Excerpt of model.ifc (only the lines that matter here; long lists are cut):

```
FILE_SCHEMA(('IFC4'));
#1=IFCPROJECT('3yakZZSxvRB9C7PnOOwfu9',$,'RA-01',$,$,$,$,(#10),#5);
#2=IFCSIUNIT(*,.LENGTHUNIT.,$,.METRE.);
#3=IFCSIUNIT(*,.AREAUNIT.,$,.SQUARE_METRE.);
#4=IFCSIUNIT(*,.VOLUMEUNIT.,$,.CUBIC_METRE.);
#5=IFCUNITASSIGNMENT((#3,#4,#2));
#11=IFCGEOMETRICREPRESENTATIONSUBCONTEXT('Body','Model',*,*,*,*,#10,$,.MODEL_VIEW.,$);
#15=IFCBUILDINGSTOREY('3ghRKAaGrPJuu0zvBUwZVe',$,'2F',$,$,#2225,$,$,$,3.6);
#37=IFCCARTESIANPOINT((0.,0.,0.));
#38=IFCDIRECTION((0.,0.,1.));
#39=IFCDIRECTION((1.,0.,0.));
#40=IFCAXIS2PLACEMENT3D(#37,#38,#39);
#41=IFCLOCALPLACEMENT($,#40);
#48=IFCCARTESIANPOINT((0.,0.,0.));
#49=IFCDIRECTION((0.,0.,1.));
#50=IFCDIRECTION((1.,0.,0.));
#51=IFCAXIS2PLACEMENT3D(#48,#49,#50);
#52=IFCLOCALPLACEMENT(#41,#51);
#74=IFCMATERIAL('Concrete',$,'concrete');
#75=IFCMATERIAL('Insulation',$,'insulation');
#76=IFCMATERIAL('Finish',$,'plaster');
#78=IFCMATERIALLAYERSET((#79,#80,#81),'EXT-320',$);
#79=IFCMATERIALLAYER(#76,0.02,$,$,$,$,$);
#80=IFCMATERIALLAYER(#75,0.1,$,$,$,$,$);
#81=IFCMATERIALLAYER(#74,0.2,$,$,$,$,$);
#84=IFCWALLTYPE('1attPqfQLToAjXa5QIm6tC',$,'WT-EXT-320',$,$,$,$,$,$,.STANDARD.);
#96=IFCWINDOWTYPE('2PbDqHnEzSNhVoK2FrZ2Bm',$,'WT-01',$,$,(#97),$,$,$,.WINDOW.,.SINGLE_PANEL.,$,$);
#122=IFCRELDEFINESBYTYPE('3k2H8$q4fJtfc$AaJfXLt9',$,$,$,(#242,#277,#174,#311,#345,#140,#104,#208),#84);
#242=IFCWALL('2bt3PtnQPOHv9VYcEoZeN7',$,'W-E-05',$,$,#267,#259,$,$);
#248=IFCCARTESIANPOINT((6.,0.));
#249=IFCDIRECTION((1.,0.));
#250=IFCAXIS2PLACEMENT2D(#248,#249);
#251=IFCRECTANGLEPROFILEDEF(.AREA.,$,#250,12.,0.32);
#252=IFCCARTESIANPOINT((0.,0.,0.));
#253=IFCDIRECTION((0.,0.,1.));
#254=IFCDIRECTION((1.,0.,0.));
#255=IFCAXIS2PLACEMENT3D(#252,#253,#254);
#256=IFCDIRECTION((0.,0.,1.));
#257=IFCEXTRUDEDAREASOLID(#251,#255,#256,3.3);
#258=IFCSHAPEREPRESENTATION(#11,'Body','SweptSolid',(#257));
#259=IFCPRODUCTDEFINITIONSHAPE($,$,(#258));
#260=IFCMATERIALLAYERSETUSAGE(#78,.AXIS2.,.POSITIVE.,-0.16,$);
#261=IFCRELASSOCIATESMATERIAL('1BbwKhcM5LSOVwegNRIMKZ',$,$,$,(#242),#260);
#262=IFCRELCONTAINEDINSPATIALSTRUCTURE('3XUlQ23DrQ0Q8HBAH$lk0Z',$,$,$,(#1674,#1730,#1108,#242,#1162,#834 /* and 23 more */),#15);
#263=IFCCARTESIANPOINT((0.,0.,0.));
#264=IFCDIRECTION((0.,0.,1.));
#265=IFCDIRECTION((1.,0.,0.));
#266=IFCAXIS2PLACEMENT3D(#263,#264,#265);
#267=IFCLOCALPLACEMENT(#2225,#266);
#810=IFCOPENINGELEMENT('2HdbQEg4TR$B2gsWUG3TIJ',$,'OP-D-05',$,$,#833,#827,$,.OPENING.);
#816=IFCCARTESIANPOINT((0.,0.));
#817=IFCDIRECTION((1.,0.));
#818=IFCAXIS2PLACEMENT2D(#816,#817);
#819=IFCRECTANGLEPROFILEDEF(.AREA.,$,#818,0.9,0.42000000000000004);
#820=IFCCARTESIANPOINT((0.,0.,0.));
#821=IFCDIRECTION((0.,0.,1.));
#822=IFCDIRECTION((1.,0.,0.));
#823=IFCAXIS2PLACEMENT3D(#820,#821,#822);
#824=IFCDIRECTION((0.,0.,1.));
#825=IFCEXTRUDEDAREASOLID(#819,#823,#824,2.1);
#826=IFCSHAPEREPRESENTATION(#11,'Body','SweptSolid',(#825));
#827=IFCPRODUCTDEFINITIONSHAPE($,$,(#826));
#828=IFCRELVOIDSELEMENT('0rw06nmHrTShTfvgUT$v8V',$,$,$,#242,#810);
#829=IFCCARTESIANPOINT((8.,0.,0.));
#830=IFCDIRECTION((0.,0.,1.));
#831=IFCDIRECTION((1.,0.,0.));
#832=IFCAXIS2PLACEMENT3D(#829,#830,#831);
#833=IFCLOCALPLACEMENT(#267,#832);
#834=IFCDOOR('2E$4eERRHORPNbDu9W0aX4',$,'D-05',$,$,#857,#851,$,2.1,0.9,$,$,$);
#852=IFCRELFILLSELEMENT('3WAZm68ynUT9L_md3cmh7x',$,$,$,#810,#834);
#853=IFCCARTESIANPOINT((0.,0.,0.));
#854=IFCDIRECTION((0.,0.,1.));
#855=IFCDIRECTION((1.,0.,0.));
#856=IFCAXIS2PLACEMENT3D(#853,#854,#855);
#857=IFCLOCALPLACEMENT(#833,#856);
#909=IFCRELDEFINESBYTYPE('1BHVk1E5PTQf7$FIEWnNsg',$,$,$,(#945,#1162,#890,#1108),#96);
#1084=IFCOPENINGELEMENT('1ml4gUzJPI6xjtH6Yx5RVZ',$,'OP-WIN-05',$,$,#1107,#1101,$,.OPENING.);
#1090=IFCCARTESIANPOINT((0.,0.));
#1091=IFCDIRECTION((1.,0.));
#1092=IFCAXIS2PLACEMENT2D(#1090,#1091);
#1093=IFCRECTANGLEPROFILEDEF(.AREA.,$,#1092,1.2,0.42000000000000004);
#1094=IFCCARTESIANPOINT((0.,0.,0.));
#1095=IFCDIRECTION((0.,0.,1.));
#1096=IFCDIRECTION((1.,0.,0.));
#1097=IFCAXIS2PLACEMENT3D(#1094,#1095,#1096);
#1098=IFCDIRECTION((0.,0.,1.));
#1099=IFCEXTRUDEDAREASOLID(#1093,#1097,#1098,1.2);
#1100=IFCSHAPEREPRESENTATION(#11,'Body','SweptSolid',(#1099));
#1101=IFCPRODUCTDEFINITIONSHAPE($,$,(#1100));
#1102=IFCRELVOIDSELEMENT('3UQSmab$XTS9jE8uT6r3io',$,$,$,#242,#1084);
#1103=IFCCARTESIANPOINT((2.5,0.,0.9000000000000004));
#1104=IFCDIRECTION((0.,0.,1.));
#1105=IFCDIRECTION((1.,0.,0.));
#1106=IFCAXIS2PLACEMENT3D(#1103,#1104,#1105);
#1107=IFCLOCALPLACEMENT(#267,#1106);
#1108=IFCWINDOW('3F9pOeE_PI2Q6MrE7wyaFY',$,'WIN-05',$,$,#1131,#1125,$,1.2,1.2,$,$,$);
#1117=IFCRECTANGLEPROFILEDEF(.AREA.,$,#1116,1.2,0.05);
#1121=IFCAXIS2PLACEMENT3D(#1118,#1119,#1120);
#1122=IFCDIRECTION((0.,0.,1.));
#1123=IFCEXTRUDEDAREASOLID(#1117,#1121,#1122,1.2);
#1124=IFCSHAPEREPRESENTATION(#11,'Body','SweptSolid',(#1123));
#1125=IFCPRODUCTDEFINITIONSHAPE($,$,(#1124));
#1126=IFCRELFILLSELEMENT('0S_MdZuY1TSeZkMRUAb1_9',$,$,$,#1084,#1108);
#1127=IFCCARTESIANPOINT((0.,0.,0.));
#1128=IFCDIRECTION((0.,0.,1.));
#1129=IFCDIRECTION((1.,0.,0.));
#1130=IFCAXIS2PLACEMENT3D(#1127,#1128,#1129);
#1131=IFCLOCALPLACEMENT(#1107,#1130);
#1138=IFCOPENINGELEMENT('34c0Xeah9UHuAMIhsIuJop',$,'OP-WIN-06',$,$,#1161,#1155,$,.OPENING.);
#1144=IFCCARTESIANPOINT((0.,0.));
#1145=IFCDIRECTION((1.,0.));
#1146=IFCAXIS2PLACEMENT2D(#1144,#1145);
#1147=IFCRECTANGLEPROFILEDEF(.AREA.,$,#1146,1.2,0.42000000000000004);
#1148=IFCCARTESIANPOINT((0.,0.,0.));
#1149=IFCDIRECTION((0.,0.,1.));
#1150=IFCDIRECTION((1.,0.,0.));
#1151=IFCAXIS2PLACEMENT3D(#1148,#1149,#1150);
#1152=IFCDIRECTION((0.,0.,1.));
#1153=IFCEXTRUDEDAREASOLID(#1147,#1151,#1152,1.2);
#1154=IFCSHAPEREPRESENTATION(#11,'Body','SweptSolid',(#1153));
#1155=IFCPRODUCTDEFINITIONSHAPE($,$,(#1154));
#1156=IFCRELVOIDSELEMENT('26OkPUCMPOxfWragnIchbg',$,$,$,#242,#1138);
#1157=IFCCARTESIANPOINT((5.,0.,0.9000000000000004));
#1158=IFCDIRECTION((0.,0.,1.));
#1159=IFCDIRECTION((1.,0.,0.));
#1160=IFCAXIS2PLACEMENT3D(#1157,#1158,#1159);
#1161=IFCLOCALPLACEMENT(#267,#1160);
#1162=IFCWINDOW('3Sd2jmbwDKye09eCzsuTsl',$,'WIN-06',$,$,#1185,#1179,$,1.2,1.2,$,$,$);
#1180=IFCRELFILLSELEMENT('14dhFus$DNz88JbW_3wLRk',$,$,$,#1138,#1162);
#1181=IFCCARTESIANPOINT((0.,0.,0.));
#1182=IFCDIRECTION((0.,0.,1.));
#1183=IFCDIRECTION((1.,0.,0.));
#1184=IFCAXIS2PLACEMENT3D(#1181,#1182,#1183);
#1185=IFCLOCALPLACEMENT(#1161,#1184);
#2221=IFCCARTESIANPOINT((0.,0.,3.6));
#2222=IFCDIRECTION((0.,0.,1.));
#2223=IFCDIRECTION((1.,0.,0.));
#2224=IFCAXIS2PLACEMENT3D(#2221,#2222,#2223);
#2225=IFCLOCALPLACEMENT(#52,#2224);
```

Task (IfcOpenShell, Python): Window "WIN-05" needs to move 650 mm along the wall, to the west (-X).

```python
import ifcopenshell
import ifcopenshell.api.geometry
import ifcopenshell.util.placement
import ifcopenshell.util.unit

model = ifcopenshell.open("model.ifc")
unit_scale = ifcopenshell.util.unit.calculate_unit_scale(model)

window = model.by_id(1108)
opening = window.FillsVoids[0].RelatingOpeningElement
wall = opening.VoidsElements[0].RelatingBuildingElement

wall_matrix = ifcopenshell.util.placement.get_local_placement(wall.ObjectPlacement)
shift = wall_matrix[:3, 0] * -0.65 / unit_scale
before = ifcopenshell.util.placement.get_local_placement(window.ObjectPlacement)[:3, 3].copy()

# The window is placed relative to its opening, so it follows when the opening moves.
matrix = ifcopenshell.util.placement.get_local_placement(opening.ObjectPlacement)
matrix[:3, 3] += shift
ifcopenshell.api.geometry.edit_object_placement(
    model, product=opening, matrix=matrix, is_si=False, should_transform_children=True
)

after = ifcopenshell.util.placement.get_local_placement(window.ObjectPlacement)[:3, 3]
print("window moved by", (after - before).round(3) + 0.0)

model.write("model_edited.ifc")
```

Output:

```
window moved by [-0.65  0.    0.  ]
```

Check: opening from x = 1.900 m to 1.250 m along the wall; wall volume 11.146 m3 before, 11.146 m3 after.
